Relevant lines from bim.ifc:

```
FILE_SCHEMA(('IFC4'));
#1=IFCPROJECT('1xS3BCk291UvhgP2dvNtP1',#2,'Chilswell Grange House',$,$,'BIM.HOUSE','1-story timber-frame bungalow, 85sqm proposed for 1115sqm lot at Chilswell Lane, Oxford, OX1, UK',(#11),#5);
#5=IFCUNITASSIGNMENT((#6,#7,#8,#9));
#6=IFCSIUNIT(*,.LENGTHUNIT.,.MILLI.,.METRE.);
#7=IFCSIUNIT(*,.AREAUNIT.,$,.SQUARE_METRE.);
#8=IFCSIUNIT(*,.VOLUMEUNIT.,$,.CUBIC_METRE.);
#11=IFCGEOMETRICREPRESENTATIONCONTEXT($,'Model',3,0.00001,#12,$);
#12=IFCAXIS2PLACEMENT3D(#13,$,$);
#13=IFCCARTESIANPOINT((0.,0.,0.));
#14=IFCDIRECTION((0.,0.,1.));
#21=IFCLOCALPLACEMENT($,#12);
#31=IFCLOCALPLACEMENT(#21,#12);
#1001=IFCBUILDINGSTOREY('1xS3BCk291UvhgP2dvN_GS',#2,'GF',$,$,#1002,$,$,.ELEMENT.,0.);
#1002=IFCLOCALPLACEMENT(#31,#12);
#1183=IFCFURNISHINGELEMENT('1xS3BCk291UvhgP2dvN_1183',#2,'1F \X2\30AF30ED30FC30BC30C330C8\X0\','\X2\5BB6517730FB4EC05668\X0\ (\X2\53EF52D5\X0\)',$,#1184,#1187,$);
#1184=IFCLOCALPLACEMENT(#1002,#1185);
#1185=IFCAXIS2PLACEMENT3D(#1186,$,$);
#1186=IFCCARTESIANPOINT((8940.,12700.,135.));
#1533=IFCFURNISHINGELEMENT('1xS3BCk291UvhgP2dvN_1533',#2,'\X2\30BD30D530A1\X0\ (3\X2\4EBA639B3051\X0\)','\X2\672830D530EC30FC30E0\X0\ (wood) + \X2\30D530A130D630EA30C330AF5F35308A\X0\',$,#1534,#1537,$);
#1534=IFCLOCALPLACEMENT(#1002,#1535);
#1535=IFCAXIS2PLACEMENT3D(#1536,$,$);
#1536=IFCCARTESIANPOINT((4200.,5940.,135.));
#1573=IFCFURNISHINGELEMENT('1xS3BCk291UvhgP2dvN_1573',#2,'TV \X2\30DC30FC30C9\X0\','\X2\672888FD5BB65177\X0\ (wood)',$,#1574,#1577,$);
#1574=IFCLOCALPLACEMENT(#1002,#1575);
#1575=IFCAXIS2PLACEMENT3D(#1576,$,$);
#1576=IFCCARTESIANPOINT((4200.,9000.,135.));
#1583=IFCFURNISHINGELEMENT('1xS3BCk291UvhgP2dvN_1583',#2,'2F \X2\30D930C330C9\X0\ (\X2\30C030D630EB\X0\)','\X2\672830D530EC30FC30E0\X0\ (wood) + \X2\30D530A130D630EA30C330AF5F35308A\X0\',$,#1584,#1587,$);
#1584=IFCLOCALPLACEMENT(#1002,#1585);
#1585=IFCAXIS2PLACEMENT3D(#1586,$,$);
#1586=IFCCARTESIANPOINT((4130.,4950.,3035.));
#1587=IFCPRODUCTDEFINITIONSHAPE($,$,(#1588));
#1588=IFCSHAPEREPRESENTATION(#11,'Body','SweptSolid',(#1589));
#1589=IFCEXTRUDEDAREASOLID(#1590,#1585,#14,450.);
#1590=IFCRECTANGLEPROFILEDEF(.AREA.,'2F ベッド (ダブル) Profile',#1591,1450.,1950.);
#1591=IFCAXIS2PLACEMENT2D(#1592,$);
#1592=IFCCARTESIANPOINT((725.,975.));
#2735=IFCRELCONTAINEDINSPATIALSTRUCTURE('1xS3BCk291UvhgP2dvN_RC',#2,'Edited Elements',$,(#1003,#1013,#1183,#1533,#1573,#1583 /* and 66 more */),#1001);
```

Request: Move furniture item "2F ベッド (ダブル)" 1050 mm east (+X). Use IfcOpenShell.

```python
import ifcopenshell
import ifcopenshell.api.geometry
import ifcopenshell.util.placement

model = ifcopenshell.open("bim.ifc")

item = model.by_guid("1xS3BCk291UvhgP2dvN_1583")
matrix = ifcopenshell.util.placement.get_local_placement(item.ObjectPlacement)
matrix[0, 3] += 1050.0
ifcopenshell.api.geometry.edit_object_placement(model, product=item, matrix=matrix, is_si=False)

print(ifcopenshell.util.placement.get_local_placement(item.ObjectPlacement).round(3) + 0.0)

model.write("bim-out.ifc")
```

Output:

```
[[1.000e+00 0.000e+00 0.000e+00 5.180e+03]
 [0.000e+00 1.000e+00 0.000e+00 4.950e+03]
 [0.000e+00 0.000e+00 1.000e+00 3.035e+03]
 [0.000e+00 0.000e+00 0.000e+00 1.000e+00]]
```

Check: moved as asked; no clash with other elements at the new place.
